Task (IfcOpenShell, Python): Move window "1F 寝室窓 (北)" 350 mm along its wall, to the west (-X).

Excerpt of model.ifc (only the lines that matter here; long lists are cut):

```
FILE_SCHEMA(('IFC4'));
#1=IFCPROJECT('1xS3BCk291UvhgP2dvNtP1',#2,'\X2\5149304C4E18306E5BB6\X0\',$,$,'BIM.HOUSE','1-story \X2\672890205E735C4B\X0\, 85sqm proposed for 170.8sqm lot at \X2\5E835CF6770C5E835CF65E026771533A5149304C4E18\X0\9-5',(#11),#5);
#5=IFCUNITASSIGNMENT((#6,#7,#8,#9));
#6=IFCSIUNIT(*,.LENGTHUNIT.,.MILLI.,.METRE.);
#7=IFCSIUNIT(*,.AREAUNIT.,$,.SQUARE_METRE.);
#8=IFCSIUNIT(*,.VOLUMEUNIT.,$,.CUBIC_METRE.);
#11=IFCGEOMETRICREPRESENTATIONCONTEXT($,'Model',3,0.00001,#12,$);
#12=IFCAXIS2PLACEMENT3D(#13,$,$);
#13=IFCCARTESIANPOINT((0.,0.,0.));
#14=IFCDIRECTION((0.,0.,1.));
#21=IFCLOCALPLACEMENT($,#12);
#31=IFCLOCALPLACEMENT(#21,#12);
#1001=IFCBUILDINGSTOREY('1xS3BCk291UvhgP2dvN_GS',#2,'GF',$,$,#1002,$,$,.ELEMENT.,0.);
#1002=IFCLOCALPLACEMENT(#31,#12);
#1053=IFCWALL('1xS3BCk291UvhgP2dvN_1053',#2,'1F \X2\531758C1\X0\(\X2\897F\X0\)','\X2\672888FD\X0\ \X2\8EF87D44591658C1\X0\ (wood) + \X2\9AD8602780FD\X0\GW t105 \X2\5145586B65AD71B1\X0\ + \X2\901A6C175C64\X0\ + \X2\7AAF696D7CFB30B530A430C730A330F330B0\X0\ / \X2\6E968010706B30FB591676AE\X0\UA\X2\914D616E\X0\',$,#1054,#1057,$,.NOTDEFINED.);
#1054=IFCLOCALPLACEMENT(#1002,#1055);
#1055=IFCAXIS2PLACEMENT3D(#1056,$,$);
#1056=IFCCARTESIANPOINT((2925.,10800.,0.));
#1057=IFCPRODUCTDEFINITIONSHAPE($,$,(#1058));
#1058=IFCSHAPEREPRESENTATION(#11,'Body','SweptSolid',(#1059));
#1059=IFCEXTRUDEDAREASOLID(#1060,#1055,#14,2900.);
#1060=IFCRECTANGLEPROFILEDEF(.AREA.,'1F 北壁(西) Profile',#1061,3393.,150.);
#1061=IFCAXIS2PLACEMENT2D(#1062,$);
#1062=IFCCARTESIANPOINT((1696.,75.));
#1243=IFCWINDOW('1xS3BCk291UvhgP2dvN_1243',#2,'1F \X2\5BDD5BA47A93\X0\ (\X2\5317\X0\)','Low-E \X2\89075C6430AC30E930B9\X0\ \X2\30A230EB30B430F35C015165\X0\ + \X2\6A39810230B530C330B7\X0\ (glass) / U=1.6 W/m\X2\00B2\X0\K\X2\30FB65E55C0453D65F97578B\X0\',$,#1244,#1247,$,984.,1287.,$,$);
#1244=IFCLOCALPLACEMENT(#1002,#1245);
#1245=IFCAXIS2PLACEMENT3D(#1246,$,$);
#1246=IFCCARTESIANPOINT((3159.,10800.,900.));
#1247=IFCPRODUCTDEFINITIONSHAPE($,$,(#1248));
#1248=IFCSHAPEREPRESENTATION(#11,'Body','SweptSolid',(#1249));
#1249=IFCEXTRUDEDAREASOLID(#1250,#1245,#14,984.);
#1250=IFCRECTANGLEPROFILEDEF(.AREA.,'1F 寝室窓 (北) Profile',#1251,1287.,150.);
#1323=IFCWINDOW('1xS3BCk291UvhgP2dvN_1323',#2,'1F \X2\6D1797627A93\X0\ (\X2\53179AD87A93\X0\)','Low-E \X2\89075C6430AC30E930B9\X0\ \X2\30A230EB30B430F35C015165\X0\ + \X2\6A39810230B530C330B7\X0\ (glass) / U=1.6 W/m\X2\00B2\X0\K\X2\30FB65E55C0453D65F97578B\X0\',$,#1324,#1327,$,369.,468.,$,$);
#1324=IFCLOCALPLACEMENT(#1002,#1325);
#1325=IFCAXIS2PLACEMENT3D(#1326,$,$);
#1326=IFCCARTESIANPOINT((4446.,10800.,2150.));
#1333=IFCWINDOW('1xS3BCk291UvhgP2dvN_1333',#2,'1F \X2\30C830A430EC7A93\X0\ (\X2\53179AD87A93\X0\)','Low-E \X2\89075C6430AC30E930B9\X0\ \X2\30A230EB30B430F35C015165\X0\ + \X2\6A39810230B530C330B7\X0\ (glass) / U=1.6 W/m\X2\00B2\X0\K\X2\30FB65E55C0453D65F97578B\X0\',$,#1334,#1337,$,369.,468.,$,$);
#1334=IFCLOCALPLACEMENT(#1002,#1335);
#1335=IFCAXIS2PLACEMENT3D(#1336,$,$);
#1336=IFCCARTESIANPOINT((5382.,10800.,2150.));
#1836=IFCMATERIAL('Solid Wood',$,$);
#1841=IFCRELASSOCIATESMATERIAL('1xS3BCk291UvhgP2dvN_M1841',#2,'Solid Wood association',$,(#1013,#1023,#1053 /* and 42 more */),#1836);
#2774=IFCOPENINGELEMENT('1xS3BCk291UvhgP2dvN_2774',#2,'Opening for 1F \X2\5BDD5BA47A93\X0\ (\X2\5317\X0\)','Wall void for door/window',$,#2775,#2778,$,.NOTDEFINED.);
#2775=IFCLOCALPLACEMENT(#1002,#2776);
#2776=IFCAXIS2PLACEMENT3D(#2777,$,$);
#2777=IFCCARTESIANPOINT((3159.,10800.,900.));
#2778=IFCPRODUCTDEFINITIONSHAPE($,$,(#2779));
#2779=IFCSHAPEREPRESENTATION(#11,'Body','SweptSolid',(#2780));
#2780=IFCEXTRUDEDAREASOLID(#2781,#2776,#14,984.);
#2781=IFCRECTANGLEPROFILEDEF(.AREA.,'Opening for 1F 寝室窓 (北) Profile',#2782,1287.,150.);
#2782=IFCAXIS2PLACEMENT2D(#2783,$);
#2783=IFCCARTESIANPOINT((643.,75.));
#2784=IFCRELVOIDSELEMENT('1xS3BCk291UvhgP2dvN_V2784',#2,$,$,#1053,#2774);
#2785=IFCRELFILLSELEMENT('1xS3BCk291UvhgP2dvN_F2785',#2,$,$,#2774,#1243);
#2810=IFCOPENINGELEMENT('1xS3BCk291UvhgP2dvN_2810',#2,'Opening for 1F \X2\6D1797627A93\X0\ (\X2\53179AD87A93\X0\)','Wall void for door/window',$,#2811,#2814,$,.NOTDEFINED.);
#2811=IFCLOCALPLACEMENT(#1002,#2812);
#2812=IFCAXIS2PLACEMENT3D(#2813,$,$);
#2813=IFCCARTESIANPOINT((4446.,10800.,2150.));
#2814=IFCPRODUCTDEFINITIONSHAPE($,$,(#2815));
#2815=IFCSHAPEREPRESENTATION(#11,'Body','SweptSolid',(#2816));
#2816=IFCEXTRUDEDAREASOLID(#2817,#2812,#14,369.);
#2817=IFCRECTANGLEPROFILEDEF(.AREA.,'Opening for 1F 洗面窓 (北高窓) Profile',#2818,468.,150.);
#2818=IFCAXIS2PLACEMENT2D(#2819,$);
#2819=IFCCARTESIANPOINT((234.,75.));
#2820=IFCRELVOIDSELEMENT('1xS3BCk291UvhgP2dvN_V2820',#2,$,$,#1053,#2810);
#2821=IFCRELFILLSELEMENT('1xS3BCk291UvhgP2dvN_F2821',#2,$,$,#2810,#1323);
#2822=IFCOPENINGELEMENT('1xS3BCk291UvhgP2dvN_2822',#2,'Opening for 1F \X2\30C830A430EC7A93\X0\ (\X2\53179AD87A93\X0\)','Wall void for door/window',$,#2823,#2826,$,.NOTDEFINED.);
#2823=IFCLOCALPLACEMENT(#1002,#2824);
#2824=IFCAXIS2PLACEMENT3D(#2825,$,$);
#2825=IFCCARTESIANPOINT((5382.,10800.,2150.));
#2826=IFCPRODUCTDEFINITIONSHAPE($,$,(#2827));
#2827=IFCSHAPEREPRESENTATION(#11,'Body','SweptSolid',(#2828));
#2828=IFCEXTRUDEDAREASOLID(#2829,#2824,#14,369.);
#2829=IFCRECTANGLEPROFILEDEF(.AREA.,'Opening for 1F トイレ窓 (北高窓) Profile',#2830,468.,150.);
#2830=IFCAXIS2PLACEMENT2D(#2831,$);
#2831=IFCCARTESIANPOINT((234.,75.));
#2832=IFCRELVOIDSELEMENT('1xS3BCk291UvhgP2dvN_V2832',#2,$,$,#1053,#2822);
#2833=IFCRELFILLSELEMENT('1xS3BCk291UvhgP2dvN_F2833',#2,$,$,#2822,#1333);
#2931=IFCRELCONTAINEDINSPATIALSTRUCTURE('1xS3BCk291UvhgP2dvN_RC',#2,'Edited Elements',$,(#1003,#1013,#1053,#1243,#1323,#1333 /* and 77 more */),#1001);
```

```python
import ifcopenshell
import ifcopenshell.api.geometry
import ifcopenshell.util.placement

model = ifcopenshell.open("model.ifc")

window = model.by_guid("1xS3BCk291UvhgP2dvN_1243")
opening = window.FillsVoids[0].RelatingOpeningElement
wall = opening.VoidsElements[0].RelatingBuildingElement

wall_matrix = ifcopenshell.util.placement.get_local_placement(wall.ObjectPlacement)
shift = wall_matrix[:3, 0] * -350.0
before = ifcopenshell.util.placement.get_local_placement(window.ObjectPlacement)[:3, 3].copy()

# The window is not placed relative to its opening, so move both.
for product in (opening, window):
    matrix = ifcopenshell.util.placement.get_local_placement(product.ObjectPlacement)
    matrix[:3, 3] += shift
    ifcopenshell.api.geometry.edit_object_placement(model, product=product, matrix=matrix, is_si=False)

after = ifcopenshell.util.placement.get_local_placement(window.ObjectPlacement)[:3, 3]
print("window moved by", (after - before).round(3) + 0.0)

model.write("model_v2.ifc")
```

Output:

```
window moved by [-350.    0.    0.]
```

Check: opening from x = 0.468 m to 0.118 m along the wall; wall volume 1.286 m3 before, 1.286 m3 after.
